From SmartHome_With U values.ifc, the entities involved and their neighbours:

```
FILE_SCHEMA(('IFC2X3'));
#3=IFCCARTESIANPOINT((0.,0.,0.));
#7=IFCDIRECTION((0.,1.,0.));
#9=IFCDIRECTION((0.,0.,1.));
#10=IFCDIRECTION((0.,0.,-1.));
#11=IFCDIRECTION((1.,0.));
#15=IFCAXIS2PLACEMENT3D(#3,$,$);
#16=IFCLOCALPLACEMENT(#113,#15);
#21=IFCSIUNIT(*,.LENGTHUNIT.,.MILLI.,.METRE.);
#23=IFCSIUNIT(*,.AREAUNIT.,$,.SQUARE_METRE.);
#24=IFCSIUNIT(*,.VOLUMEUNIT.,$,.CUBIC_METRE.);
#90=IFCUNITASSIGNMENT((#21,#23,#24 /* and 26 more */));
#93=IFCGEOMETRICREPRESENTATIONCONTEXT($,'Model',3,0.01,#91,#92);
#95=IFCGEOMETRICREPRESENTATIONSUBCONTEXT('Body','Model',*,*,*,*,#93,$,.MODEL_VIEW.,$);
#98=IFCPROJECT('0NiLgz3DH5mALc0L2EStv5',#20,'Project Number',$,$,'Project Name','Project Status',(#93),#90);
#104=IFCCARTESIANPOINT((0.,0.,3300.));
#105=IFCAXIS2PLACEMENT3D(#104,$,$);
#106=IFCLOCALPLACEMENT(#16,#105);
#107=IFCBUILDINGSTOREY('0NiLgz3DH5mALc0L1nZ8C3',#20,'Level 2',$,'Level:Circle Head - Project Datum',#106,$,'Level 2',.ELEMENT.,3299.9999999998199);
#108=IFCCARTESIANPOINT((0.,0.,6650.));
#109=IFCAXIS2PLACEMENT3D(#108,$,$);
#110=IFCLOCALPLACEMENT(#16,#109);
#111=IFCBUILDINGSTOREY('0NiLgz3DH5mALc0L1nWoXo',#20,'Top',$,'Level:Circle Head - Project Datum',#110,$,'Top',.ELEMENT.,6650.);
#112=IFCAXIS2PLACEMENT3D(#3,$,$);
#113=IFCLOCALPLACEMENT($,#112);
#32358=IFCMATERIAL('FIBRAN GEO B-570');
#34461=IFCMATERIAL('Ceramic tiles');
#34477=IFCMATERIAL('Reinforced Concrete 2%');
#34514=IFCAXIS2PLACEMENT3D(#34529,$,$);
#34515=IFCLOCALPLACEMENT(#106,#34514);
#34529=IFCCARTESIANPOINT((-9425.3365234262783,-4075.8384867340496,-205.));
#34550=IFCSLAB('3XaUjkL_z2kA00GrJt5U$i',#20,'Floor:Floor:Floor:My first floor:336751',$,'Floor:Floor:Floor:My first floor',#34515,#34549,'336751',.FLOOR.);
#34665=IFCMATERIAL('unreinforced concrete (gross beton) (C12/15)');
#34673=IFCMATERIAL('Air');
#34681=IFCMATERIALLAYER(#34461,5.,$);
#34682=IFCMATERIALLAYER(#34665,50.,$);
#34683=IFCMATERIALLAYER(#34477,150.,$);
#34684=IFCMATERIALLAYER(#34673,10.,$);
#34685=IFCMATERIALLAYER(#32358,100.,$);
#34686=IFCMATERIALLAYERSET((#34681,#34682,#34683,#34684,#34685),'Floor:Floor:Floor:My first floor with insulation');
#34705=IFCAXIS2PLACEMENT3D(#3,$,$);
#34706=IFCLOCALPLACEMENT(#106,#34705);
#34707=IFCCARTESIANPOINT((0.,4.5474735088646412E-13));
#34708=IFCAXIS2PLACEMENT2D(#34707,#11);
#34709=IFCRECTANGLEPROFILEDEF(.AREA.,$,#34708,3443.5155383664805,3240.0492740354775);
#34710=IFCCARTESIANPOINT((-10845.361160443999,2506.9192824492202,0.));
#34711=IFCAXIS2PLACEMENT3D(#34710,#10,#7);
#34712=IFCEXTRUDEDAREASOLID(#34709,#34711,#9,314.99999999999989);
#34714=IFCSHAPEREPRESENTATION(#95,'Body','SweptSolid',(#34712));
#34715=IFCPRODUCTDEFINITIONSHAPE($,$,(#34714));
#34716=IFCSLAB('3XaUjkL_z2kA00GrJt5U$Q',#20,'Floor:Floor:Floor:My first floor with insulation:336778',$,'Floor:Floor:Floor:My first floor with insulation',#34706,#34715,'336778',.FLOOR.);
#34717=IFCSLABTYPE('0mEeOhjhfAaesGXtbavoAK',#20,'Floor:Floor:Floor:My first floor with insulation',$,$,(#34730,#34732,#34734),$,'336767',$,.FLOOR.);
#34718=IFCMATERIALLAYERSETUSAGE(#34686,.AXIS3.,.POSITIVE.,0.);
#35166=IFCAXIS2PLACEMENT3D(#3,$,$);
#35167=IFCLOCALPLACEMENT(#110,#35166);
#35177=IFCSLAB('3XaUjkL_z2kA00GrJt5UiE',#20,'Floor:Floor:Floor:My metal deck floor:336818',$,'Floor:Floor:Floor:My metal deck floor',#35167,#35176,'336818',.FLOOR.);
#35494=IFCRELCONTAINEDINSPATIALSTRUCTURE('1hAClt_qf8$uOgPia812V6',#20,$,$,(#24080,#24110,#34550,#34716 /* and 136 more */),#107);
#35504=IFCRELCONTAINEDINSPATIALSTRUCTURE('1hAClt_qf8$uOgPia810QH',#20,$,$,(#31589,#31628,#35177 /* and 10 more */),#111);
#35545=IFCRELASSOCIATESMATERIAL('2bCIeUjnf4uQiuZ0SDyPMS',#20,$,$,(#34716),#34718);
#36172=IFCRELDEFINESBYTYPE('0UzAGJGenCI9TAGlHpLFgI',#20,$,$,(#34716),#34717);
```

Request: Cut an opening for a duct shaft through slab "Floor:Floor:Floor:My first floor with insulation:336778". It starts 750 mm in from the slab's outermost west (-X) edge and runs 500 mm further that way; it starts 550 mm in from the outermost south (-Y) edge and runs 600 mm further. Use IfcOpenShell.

```python
import numpy as np
import ifcopenshell
import ifcopenshell.api.feature
import ifcopenshell.api.geometry
import ifcopenshell.api.root
import ifcopenshell.geom
import ifcopenshell.util.placement
import ifcopenshell.util.representation
import ifcopenshell.util.shape
import ifcopenshell.util.unit

model = ifcopenshell.open("SmartHome_With U values.ifc")
unit_scale = ifcopenshell.util.unit.calculate_unit_scale(model)
settings = ifcopenshell.geom.settings()


def volume(element):
    """Net volume in cubic metres, openings subtracted."""
    shape = ifcopenshell.geom.create_shape(settings, element)
    return ifcopenshell.util.shape.get_volume(shape.geometry)


slab = model.by_guid("3XaUjkL_z2kA00GrJt5U$Q")
before = volume(slab)

# Extent in the slab's own axes, in metres. The edges named are its -X and -Y sides.
slab_shape = ifcopenshell.geom.create_shape(settings, slab)
vertices = ifcopenshell.util.shape.get_vertices(slab_shape.geometry)
x_min, y_min, bottom = vertices.min(axis=0)
top = vertices[:, 2].max()

opening = ifcopenshell.api.root.create_entity(model, ifc_class="IfcOpeningElement", name="Duct shaft opening")
context = ifcopenshell.util.representation.get_context(model, "Model", "Body", "MODEL_VIEW")
width, depth = 0.5, 0.6
outline = [(0.0, 0.0), (width, 0.0), (width, depth), (0.0, depth), (0.0, 0.0)]
# Overshoot both faces by 50 mm so the cut is clean.
shape = ifcopenshell.api.geometry.add_slab_representation(
    model, context=context, depth=top - bottom + 0.1, polyline=outline
)
ifcopenshell.api.geometry.assign_representation(model, product=opening, representation=shape)

matrix = ifcopenshell.util.placement.get_local_placement(slab.ObjectPlacement)
matrix[:, 3] = matrix @ np.append(np.array([x_min + 0.75, y_min + 0.55, bottom - 0.05]) / unit_scale, 1.0)
ifcopenshell.api.geometry.edit_object_placement(model, product=opening, matrix=matrix, is_si=False)
ifcopenshell.api.feature.add_feature(model, feature=opening, element=slab)

after = volume(slab)

print(f"slab volume {before:.3f} -> {after:.3f} m3")

model.write("SmartHome_With U values_v2.ifc")
```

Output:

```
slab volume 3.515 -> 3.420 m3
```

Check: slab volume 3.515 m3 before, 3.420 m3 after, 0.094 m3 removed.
